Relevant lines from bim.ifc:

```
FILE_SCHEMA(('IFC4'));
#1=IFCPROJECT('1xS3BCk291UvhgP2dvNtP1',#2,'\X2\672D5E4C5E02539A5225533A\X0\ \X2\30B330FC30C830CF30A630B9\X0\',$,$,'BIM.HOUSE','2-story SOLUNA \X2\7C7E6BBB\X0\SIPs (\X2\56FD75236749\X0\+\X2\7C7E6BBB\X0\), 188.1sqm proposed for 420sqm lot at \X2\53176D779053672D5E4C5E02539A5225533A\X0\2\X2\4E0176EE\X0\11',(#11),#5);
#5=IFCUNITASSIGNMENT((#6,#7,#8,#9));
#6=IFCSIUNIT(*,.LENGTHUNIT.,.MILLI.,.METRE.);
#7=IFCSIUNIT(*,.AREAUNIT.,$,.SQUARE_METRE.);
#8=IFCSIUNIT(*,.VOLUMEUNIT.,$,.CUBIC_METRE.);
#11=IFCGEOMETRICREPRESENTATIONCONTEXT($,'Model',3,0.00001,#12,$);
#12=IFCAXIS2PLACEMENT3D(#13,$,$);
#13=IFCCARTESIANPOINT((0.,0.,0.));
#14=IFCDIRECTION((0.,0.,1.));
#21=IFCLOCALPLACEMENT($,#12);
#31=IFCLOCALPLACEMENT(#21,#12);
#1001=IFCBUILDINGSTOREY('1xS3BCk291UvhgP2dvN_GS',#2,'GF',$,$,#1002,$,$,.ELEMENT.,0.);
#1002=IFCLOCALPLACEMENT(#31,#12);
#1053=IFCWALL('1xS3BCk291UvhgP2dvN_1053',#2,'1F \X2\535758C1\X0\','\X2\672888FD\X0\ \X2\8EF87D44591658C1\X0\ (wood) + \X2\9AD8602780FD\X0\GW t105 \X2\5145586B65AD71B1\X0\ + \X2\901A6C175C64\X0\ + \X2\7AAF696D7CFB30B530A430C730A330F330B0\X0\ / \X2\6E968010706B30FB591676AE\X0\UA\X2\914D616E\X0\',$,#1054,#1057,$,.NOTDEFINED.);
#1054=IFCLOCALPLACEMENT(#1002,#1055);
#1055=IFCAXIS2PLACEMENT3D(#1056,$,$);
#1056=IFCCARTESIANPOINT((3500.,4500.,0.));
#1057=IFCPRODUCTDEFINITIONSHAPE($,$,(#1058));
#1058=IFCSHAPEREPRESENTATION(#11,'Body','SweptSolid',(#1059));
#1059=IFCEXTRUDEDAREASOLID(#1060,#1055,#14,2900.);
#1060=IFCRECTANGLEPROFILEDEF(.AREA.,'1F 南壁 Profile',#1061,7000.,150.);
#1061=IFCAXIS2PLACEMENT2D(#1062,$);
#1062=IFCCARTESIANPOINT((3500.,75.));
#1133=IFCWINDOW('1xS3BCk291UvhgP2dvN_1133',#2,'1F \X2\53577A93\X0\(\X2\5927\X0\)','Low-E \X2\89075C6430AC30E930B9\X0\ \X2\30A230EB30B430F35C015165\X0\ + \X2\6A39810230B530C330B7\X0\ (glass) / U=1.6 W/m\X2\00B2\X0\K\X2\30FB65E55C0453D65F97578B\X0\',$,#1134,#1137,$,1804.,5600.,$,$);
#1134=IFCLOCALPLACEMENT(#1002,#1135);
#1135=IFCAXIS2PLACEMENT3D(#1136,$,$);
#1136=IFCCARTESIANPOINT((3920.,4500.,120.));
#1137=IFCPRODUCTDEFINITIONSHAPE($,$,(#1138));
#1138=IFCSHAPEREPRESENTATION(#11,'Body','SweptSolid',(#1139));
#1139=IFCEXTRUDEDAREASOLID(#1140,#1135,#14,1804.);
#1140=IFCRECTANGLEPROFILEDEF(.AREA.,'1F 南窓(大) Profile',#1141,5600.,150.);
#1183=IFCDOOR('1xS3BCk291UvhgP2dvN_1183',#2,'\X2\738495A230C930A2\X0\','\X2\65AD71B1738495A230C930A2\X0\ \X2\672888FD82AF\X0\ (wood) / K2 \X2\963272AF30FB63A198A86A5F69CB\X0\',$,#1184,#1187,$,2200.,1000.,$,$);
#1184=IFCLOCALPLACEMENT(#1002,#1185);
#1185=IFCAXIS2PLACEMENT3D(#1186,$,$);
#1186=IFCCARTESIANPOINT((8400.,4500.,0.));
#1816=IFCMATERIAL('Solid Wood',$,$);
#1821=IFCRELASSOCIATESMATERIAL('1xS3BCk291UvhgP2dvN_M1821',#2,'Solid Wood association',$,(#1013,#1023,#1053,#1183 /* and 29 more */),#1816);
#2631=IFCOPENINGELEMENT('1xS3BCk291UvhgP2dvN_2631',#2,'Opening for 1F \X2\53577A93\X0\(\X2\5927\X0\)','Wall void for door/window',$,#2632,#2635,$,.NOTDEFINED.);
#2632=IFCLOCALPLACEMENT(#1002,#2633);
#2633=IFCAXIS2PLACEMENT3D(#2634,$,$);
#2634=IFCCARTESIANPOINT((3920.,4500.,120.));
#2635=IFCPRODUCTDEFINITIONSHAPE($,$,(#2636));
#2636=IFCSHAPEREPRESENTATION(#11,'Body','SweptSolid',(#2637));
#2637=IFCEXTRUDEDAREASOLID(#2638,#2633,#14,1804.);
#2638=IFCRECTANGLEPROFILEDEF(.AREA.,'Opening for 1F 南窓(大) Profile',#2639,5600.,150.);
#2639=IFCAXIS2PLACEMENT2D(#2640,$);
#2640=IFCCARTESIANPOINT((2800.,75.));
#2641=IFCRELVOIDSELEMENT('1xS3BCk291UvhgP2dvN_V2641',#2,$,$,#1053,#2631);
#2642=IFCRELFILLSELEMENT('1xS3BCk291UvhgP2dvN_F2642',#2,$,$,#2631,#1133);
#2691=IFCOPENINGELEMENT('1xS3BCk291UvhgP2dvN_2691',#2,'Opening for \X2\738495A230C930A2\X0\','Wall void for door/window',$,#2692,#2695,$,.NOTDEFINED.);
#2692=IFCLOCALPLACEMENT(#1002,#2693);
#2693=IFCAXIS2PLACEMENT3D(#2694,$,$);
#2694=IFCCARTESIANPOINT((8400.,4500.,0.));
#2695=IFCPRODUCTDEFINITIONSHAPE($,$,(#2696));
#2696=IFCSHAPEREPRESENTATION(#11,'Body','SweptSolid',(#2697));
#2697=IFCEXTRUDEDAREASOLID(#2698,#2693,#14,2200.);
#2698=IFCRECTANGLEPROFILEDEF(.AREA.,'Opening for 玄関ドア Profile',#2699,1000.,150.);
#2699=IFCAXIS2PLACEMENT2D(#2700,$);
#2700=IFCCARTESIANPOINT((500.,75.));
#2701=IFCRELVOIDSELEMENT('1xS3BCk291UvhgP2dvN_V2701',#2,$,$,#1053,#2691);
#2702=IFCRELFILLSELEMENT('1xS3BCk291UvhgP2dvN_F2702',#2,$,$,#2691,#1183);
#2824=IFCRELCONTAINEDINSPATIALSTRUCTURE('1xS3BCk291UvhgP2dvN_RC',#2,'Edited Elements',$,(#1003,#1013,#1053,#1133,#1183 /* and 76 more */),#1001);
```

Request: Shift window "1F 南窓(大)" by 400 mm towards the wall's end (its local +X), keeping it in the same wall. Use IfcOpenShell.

```python
import ifcopenshell
import ifcopenshell.api.geometry
import ifcopenshell.util.placement
import ifcopenshell.util.unit

model = ifcopenshell.open("bim.ifc")
unit_scale = ifcopenshell.util.unit.calculate_unit_scale(model)

window = model.by_id(1133)
opening = window.FillsVoids[0].RelatingOpeningElement
wall = opening.VoidsElements[0].RelatingBuildingElement

wall_matrix = ifcopenshell.util.placement.get_local_placement(wall.ObjectPlacement)
shift = wall_matrix[:3, 0] * 0.4 / unit_scale
before = ifcopenshell.util.placement.get_local_placement(window.ObjectPlacement)[:3, 3].copy()

# The window is not placed relative to its opening, so move both.
for product in (opening, window):
    matrix = ifcopenshell.util.placement.get_local_placement(product.ObjectPlacement)
    matrix[:3, 3] += shift
    ifcopenshell.api.geometry.edit_object_placement(model, product=product, matrix=matrix, is_si=False)

after = ifcopenshell.util.placement.get_local_placement(window.ObjectPlacement)[:3, 3]
print("window moved by", (after - before).round(3) + 0.0)

model.write("bim_v2.ifc")
```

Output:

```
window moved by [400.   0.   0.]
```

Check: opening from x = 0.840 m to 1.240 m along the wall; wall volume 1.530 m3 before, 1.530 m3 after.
